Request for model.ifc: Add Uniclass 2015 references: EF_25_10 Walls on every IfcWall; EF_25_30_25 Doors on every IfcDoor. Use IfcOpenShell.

First a look at what the model holds.

```python
import ifcopenshell

model = ifcopenshell.open("model.ifc")
print(model.schema)
print("classifications:", [c.Name for c in model.by_type("IfcClassification")])
for ifc_class in ("IfcDoor", "IfcRoof", "IfcStair", "IfcWall", "IfcWindow"):
    print(ifc_class, len(model.by_type(ifc_class)))
```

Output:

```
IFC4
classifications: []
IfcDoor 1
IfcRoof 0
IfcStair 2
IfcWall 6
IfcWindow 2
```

```python
import ifcopenshell
import ifcopenshell.api.classification

model = ifcopenshell.open("model.ifc")

system = ifcopenshell.api.classification.add_classification(model, classification="Uniclass 2015")

codes = {
    "IfcWall": ("EF_25_10", "Walls"),
    "IfcDoor": ("EF_25_30_25", "Doors"),
}
for ifc_class, (code, name) in codes.items():
    products = model.by_type(ifc_class)
    ifcopenshell.api.classification.add_reference(
        model, products=products, classification=system, identification=code, name=name
    )
    print(code, len(products))

model.write("model_rev.ifc")
```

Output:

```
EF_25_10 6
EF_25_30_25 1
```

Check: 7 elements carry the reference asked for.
